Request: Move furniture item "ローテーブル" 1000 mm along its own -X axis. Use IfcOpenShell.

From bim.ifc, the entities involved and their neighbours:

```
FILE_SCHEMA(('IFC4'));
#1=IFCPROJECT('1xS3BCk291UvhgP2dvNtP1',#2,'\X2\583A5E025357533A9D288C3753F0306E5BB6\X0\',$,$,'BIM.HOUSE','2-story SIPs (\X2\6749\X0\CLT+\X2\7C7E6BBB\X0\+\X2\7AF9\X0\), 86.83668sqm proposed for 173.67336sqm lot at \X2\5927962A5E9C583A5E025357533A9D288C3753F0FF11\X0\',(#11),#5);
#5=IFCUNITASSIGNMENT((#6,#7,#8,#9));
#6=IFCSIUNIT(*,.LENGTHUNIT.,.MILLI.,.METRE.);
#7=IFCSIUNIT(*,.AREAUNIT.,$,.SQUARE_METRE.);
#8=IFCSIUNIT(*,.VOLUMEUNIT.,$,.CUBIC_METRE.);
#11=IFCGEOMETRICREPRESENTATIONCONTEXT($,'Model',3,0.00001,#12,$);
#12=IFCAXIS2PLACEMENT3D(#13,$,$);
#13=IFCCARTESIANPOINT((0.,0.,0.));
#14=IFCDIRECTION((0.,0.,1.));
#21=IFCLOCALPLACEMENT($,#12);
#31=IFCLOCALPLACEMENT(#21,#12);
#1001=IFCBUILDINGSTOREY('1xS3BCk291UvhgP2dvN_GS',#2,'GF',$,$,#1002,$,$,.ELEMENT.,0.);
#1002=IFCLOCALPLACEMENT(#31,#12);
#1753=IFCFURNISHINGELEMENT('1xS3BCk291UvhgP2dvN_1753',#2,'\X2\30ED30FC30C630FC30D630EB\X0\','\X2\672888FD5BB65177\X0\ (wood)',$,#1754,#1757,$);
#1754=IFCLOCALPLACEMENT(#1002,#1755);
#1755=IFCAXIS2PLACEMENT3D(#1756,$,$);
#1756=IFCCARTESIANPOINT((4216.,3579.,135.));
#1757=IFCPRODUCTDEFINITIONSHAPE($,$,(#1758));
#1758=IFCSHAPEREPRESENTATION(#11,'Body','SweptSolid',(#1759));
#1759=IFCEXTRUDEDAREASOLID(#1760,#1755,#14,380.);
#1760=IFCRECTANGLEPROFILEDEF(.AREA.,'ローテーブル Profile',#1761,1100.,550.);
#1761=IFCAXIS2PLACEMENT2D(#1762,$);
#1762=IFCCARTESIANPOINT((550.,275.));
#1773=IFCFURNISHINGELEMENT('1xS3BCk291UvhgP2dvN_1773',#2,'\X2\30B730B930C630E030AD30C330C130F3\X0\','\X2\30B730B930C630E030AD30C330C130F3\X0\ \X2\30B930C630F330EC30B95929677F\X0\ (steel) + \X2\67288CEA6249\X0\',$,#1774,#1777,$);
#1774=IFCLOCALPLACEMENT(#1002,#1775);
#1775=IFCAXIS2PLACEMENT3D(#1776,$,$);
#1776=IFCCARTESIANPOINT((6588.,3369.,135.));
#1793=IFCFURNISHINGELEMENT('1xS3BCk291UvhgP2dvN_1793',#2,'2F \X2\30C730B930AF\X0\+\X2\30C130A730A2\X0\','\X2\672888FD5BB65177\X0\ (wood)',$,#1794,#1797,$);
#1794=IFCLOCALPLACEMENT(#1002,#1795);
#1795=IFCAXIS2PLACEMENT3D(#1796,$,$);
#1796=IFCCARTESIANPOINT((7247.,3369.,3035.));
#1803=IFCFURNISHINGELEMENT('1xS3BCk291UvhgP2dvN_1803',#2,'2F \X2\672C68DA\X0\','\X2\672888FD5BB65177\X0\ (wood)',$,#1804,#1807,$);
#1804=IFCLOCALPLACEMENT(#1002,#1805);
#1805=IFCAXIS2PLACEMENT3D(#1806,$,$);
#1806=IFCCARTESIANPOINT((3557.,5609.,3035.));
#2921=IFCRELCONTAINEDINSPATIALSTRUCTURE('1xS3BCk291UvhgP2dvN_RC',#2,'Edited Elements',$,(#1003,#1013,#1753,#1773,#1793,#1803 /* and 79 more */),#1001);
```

```python
import ifcopenshell
import ifcopenshell.api.geometry
import ifcopenshell.util.placement

model = ifcopenshell.open("bim.ifc")

item = model.by_guid("1xS3BCk291UvhgP2dvN_1753")
matrix = ifcopenshell.util.placement.get_local_placement(item.ObjectPlacement)
matrix[:3, 3] -= matrix[:3, 0] * 1000.0
ifcopenshell.api.geometry.edit_object_placement(model, product=item, matrix=matrix, is_si=False)

print(ifcopenshell.util.placement.get_local_placement(item.ObjectPlacement).round(3) + 0.0)

model.write("bim-out.ifc")
```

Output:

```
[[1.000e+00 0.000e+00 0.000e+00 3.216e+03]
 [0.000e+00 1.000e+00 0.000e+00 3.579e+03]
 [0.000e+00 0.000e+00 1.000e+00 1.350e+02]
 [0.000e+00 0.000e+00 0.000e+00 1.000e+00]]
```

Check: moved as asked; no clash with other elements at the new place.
